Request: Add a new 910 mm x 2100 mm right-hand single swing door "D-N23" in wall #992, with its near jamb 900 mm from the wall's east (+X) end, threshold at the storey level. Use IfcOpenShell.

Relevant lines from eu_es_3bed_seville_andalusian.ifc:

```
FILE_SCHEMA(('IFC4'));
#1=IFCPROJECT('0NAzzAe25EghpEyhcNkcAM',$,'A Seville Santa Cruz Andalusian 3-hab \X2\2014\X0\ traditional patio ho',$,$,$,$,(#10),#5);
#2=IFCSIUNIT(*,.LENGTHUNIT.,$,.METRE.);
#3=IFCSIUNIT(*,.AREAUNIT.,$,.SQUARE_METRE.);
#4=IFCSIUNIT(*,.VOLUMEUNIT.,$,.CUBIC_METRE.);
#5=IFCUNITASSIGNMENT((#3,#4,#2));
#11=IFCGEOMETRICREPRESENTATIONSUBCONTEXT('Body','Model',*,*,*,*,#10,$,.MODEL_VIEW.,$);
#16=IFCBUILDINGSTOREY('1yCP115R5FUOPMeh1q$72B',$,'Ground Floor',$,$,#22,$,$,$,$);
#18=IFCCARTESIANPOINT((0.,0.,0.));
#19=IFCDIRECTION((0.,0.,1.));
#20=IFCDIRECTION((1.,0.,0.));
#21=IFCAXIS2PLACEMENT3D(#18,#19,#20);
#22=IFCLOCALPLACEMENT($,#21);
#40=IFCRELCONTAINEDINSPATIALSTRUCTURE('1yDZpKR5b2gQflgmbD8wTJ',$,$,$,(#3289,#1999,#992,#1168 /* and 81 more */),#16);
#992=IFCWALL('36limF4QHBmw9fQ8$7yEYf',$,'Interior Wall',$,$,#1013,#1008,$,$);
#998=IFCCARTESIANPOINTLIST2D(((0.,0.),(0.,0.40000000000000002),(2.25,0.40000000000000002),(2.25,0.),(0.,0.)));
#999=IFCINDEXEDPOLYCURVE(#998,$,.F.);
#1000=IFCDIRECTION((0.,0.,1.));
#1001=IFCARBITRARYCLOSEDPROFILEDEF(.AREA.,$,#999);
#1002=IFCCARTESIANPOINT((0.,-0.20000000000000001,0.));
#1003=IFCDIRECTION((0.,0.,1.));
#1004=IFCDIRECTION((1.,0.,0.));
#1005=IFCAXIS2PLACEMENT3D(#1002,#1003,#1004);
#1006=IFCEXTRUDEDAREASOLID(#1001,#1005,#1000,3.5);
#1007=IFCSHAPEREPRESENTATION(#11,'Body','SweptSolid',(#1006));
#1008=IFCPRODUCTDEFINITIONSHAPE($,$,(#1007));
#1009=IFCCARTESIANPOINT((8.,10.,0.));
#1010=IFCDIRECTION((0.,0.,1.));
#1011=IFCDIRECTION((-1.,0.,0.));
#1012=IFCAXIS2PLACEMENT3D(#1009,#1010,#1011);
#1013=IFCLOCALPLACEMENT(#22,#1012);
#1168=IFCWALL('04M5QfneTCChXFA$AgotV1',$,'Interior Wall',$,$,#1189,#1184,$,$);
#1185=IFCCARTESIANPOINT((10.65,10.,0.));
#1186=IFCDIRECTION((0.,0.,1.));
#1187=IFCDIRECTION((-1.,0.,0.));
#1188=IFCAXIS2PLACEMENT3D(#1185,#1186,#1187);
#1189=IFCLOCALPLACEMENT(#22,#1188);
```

```python
import numpy as np
import ifcopenshell
import ifcopenshell.api.feature
import ifcopenshell.api.geometry
import ifcopenshell.api.root
import ifcopenshell.api.spatial
import ifcopenshell.geom
import ifcopenshell.util.element
import ifcopenshell.util.placement
import ifcopenshell.util.representation
import ifcopenshell.util.shape
import ifcopenshell.util.unit

model = ifcopenshell.open("eu_es_3bed_seville_andalusian.ifc")
unit_scale = ifcopenshell.util.unit.calculate_unit_scale(model)
settings = ifcopenshell.geom.settings()


def volume(element):
    """Net volume in cubic metres, openings subtracted."""
    shape = ifcopenshell.geom.create_shape(settings, element)
    return ifcopenshell.util.shape.get_volume(shape.geometry)


wall = model.by_guid("36limF4QHBmw9fQ8$7yEYf")
storey = ifcopenshell.util.element.get_container(wall, ifc_class="IfcBuildingStorey")
context = ifcopenshell.util.representation.get_context(model, "Model", "Body", "MODEL_VIEW")
before = volume(wall)

width, height, from_end, sill = 0.91, 2.1, 0.9, 0.0  # metres

# The wall runs along its own X axis, and the end named is its -X end.
wall_shape = ifcopenshell.geom.create_shape(settings, wall)
x, y, z = ifcopenshell.util.shape.get_vertices(wall_shape.geometry).T
start = x.min() + from_end
face, thickness = float(y.min()), float(y.max() - y.min())
wall_matrix = ifcopenshell.util.placement.get_local_placement(wall.ObjectPlacement)
level = ifcopenshell.util.placement.get_local_placement(storey.ObjectPlacement)[2, 3]


def in_wall(x, y):
    """Placement at x, y metres in the wall's axes, at sill height."""
    matrix = wall_matrix.copy()
    matrix[:, 3] = wall_matrix @ np.array([x / unit_scale, y / unit_scale, 0.0, 1.0])
    matrix[2, 3] = level + sill / unit_scale
    return matrix


# Opening: a box that overshoots both wall faces by 50 mm.
opening = ifcopenshell.api.root.create_entity(model, ifc_class="IfcOpeningElement", predefined_type="OPENING")
box = ifcopenshell.api.geometry.add_wall_representation(
    model, context=context, length=width, height=height, thickness=thickness + 0.1
)
ifcopenshell.api.geometry.assign_representation(model, product=opening, representation=box)
ifcopenshell.api.geometry.edit_object_placement(model, product=opening, matrix=in_wall(start, face - 0.05), is_si=False)
ifcopenshell.api.feature.add_feature(model, feature=opening, element=wall)

door = ifcopenshell.api.root.create_entity(model, ifc_class="IfcDoor", name="D-N23", predefined_type="DOOR")
door.OverallWidth, door.OverallHeight = width / unit_scale, height / unit_scale
door.OperationType = "SINGLE_SWING_RIGHT"
body = ifcopenshell.api.geometry.add_door_representation(
    model,
    context=context,
    overall_width=door.OverallWidth,
    overall_height=door.OverallHeight,
    operation_type="SINGLE_SWING_RIGHT",
    lining_properties={"LiningDepth": thickness / unit_scale, "ThresholdDepth": thickness / unit_scale},
)
ifcopenshell.api.geometry.assign_representation(model, product=door, representation=body)
ifcopenshell.api.spatial.assign_container(model, products=[door], relating_structure=storey)
ifcopenshell.api.feature.add_filling(model, opening=opening, element=door)

# The lining spans the wall, so the door starts at the wall face.
ifcopenshell.api.geometry.edit_object_placement(model, product=door, matrix=in_wall(start, face), is_si=False)

after = volume(wall)

print(f"wall volume {before:.3f} -> {after:.3f} m3")

model.write("eu_es_3bed_seville_andalusian_v2.ifc")
```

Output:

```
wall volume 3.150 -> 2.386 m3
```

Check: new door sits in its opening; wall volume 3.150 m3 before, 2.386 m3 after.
